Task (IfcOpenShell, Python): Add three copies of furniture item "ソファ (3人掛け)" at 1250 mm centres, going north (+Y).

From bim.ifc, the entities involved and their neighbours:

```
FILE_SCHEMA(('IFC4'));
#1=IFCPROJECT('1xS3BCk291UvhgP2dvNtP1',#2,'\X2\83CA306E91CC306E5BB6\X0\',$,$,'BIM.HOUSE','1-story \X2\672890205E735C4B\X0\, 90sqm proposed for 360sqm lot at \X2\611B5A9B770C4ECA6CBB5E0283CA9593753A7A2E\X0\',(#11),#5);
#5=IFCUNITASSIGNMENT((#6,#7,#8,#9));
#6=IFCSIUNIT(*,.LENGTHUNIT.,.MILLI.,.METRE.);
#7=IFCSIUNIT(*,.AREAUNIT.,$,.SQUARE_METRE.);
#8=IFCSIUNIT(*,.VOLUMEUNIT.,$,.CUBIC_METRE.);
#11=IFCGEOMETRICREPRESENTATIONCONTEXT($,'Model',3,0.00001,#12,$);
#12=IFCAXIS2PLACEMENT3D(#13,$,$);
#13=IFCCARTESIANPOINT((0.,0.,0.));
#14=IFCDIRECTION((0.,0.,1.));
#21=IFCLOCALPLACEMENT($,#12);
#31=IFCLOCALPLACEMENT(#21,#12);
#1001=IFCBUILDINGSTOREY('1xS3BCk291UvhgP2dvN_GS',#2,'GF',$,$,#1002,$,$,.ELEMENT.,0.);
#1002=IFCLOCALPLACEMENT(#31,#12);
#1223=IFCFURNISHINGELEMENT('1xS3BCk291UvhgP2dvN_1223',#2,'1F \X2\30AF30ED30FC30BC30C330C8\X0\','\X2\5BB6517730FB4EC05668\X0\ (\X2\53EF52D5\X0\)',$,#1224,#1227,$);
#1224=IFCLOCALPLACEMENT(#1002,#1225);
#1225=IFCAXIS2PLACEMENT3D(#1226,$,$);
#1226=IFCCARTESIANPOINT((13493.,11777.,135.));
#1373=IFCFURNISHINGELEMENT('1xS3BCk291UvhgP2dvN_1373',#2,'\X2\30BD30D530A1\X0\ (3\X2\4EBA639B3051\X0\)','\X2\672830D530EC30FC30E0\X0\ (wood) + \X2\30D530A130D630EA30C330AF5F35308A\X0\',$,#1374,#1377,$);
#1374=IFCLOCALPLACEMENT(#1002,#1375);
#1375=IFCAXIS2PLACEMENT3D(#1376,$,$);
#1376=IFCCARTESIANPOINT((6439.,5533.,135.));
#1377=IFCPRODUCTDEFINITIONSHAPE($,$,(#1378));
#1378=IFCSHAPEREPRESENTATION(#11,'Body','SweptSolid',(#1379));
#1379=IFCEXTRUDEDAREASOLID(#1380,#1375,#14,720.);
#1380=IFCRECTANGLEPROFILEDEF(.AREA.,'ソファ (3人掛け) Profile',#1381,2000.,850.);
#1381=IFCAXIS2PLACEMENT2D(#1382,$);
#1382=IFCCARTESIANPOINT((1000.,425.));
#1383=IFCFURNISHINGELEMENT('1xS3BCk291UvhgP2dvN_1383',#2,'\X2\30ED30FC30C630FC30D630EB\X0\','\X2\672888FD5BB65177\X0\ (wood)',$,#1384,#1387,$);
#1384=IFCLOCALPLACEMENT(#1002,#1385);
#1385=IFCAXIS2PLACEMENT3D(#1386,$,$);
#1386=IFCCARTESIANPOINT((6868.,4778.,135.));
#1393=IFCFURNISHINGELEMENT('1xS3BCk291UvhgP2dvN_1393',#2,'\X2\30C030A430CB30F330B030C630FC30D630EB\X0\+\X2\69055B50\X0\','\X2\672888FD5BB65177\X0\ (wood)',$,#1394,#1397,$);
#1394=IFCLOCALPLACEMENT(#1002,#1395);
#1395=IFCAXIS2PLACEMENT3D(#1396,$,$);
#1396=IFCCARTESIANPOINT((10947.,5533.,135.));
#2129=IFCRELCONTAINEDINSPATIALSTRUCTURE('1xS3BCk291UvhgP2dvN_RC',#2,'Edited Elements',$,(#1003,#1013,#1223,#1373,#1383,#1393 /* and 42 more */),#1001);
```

```python
import numpy as np
import ifcopenshell
import ifcopenshell.api.geometry
import ifcopenshell.api.root
import ifcopenshell.util.element
import ifcopenshell.util.placement
import ifcopenshell.util.unit

model = ifcopenshell.open("bim.ifc")
unit_scale = ifcopenshell.util.unit.calculate_unit_scale(model)


def reuse_history(source, copy):
    """copy_class also copies each property set's owner history, people and application; keep the originals."""
    for rel in copy.IsDefinedBy:
        if rel.is_a("IfcRelDefinesByProperties") and (history := rel.RelatingPropertyDefinition.OwnerHistory):
            rel.RelatingPropertyDefinition.OwnerHistory = source.OwnerHistory
            ifcopenshell.util.element.remove_deep2(model, history)


source = model.by_id(1373)
base = ifcopenshell.util.placement.get_local_placement(source.ObjectPlacement)
step = np.array([0.0, 1.0, 0.0]) * 1.25 / unit_scale

for i in range(1, 4):
    copy = ifcopenshell.api.root.copy_class(model, product=source)
    copy.Representation = ifcopenshell.util.element.copy_deep(
        model, source.Representation, exclude=["IfcGeometricRepresentationContext", "IfcRepresentationMap"]
    )
    reuse_history(source, copy)
    matrix = base.copy()
    matrix[:3, 3] += i * step
    print("added at", matrix[:3, 3].round(3) + 0.0)
    ifcopenshell.api.geometry.edit_object_placement(model, product=copy, matrix=matrix, is_si=False)

model.write("bim_edited.ifc")
```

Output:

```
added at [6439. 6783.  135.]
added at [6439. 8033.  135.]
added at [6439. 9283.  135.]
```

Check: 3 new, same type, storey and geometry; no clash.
